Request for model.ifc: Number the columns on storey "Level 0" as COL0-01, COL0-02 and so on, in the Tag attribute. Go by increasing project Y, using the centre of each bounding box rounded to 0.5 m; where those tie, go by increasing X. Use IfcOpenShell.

First a look at what the model holds.

```python
import ifcopenshell
import ifcopenshell.util.element
import ifcopenshell.util.placement

model = ifcopenshell.open("model.ifc")
print(model.schema)
storey = next(s for s in model.by_type("IfcBuildingStorey") if s.Name == "Level 0")
columns = [e for e in ifcopenshell.util.element.get_decomposition(storey) if e.is_a("IfcColumn")]
for e in sorted(columns, key=lambda e: e.id()):
    origin = ifcopenshell.util.placement.get_local_placement(e.ObjectPlacement)[:3, 3]
    print(e.id(), e.Tag, e.Name, origin.round(2) + 0.0, sep=" | ")
```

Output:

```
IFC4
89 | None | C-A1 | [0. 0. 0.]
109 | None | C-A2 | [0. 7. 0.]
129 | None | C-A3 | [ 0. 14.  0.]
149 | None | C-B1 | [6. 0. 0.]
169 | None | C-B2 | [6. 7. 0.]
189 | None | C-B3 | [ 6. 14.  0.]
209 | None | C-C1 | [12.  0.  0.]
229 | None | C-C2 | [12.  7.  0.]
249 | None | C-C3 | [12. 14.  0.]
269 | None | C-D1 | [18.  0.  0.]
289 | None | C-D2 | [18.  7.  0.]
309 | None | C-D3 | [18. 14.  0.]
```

```python
import ifcopenshell
import ifcopenshell.geom
import ifcopenshell.util.element
import ifcopenshell.util.shape

model = ifcopenshell.open("model.ifc")
settings = ifcopenshell.geom.settings()
settings.set("use-world-coords", True)


def centre(element):
    shape = ifcopenshell.geom.create_shape(settings, element)
    return ifcopenshell.util.shape.get_bbox_centroid(shape.geometry)


storey = next(s for s in model.by_type("IfcBuildingStorey") if s.Name == "Level 0")
columns = [e for e in ifcopenshell.util.element.get_decomposition(storey) if e.is_a("IfcColumn")]

# Insertion points can sit at a corner or the storey origin, so sort by the geometry (in metres).
centres = {e: centre(e) for e in columns}
columns.sort(key=lambda e: (round(centres[e][1] / 0.5), centres[e][0]))

for i, e in enumerate(columns, start=1):
    number = f"COL0-{i:02d}"
    e.Tag = number
    print(e.id(), number)

model.write("model_rev.ifc")
```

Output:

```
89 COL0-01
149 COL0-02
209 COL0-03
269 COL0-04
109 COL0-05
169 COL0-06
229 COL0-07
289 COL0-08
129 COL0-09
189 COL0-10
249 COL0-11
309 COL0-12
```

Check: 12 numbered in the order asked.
